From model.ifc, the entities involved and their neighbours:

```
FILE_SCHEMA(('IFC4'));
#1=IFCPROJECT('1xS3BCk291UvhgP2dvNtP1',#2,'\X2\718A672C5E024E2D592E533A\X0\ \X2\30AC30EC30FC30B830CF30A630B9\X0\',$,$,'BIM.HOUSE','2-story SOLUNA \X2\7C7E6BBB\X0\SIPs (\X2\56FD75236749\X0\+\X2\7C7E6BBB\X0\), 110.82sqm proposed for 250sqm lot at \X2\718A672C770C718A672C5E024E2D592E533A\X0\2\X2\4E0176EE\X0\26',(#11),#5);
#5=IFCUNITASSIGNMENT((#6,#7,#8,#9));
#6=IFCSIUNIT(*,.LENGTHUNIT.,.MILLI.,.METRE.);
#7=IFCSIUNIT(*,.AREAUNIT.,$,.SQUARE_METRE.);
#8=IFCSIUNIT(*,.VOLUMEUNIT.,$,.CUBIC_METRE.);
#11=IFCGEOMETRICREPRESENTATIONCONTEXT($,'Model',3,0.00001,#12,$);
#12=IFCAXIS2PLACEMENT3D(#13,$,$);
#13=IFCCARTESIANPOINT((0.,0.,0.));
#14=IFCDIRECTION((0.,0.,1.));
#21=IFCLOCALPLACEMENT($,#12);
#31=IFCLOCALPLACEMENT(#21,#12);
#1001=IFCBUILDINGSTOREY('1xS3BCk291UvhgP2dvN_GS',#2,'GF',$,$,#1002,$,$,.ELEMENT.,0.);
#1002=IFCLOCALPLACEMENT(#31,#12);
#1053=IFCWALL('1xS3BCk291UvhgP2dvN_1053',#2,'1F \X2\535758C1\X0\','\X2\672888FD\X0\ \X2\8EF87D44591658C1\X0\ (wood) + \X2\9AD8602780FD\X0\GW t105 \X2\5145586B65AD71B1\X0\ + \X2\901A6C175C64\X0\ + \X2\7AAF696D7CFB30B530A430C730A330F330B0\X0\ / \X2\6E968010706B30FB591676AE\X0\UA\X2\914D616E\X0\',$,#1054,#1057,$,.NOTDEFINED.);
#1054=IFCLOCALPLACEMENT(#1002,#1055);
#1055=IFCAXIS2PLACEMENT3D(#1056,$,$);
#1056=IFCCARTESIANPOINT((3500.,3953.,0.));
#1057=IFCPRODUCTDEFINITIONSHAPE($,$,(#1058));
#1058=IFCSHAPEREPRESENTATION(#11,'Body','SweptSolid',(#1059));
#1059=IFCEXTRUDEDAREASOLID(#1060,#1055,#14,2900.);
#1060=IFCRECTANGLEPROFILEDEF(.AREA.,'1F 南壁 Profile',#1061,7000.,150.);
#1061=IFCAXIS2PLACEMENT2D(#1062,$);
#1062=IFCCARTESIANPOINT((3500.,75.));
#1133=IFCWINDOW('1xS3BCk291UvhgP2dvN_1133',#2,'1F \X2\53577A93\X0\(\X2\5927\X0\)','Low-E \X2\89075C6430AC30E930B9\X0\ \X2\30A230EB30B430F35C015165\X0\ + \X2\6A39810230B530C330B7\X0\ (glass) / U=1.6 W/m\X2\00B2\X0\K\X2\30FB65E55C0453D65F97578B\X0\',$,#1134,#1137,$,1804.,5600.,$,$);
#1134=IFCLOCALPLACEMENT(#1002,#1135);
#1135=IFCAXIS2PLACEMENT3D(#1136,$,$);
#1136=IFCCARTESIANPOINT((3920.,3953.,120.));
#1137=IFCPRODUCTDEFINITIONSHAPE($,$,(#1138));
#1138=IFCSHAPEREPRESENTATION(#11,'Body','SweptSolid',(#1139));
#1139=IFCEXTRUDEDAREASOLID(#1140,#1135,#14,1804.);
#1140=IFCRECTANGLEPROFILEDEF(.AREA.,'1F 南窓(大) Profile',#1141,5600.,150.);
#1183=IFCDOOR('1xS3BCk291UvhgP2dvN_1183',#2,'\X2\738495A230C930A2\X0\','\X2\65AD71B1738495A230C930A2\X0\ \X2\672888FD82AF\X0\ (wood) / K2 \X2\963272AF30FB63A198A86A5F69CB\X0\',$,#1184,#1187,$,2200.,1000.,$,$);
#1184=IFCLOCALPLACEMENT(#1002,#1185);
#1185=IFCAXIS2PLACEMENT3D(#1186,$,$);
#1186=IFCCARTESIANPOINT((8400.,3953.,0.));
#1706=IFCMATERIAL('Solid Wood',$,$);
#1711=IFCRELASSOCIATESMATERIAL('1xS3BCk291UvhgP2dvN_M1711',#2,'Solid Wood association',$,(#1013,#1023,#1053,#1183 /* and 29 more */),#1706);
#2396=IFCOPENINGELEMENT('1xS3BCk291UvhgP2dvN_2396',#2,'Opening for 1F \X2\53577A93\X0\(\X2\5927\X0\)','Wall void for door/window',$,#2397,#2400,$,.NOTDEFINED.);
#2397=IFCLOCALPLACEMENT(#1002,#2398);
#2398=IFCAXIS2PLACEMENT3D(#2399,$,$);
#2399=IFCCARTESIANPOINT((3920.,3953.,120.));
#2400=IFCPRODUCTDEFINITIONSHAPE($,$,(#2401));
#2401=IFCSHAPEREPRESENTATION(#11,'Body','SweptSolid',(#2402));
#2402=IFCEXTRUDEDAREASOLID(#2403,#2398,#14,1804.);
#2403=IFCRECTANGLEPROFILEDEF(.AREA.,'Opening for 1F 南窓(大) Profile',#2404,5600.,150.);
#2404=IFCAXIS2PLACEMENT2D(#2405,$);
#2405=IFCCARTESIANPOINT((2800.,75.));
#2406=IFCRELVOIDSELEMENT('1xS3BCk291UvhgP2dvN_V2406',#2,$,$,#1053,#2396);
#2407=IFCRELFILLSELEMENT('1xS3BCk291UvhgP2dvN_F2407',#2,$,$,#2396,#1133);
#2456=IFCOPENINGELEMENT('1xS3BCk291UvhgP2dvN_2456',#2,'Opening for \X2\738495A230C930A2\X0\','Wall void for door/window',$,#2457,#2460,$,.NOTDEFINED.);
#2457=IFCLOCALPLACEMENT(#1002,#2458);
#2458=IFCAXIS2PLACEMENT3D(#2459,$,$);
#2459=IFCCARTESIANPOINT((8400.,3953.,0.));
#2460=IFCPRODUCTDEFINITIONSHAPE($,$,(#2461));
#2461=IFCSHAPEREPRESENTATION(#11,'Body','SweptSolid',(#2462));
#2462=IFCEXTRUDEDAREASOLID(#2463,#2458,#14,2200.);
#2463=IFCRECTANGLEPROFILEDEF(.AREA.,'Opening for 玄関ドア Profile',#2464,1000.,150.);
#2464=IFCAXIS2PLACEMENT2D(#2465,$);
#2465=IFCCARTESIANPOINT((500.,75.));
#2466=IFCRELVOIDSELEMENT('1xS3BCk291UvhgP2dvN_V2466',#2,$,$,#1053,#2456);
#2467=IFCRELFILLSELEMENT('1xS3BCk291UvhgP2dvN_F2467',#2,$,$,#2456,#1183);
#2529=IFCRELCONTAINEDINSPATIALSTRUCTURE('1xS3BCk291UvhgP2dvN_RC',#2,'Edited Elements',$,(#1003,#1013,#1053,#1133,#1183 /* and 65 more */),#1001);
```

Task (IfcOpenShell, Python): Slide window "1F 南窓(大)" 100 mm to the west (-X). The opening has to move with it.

```python
import ifcopenshell
import ifcopenshell.api.geometry
import ifcopenshell.util.placement
import ifcopenshell.util.unit

model = ifcopenshell.open("model.ifc")
unit_scale = ifcopenshell.util.unit.calculate_unit_scale(model)

window = model.by_id(1133)
opening = window.FillsVoids[0].RelatingOpeningElement
wall = opening.VoidsElements[0].RelatingBuildingElement

wall_matrix = ifcopenshell.util.placement.get_local_placement(wall.ObjectPlacement)
shift = wall_matrix[:3, 0] * -0.1 / unit_scale
before = ifcopenshell.util.placement.get_local_placement(window.ObjectPlacement)[:3, 3].copy()

# The window is not placed relative to its opening, so move both.
for product in (opening, window):
    matrix = ifcopenshell.util.placement.get_local_placement(product.ObjectPlacement)
    matrix[:3, 3] += shift
    ifcopenshell.api.geometry.edit_object_placement(model, product=product, matrix=matrix, is_si=False)

after = ifcopenshell.util.placement.get_local_placement(window.ObjectPlacement)[:3, 3]
print("window moved by", (after - before).round(3) + 0.0)

model.write("model-out.ifc")
```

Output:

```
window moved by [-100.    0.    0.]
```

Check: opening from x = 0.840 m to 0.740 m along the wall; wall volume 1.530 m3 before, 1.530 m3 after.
